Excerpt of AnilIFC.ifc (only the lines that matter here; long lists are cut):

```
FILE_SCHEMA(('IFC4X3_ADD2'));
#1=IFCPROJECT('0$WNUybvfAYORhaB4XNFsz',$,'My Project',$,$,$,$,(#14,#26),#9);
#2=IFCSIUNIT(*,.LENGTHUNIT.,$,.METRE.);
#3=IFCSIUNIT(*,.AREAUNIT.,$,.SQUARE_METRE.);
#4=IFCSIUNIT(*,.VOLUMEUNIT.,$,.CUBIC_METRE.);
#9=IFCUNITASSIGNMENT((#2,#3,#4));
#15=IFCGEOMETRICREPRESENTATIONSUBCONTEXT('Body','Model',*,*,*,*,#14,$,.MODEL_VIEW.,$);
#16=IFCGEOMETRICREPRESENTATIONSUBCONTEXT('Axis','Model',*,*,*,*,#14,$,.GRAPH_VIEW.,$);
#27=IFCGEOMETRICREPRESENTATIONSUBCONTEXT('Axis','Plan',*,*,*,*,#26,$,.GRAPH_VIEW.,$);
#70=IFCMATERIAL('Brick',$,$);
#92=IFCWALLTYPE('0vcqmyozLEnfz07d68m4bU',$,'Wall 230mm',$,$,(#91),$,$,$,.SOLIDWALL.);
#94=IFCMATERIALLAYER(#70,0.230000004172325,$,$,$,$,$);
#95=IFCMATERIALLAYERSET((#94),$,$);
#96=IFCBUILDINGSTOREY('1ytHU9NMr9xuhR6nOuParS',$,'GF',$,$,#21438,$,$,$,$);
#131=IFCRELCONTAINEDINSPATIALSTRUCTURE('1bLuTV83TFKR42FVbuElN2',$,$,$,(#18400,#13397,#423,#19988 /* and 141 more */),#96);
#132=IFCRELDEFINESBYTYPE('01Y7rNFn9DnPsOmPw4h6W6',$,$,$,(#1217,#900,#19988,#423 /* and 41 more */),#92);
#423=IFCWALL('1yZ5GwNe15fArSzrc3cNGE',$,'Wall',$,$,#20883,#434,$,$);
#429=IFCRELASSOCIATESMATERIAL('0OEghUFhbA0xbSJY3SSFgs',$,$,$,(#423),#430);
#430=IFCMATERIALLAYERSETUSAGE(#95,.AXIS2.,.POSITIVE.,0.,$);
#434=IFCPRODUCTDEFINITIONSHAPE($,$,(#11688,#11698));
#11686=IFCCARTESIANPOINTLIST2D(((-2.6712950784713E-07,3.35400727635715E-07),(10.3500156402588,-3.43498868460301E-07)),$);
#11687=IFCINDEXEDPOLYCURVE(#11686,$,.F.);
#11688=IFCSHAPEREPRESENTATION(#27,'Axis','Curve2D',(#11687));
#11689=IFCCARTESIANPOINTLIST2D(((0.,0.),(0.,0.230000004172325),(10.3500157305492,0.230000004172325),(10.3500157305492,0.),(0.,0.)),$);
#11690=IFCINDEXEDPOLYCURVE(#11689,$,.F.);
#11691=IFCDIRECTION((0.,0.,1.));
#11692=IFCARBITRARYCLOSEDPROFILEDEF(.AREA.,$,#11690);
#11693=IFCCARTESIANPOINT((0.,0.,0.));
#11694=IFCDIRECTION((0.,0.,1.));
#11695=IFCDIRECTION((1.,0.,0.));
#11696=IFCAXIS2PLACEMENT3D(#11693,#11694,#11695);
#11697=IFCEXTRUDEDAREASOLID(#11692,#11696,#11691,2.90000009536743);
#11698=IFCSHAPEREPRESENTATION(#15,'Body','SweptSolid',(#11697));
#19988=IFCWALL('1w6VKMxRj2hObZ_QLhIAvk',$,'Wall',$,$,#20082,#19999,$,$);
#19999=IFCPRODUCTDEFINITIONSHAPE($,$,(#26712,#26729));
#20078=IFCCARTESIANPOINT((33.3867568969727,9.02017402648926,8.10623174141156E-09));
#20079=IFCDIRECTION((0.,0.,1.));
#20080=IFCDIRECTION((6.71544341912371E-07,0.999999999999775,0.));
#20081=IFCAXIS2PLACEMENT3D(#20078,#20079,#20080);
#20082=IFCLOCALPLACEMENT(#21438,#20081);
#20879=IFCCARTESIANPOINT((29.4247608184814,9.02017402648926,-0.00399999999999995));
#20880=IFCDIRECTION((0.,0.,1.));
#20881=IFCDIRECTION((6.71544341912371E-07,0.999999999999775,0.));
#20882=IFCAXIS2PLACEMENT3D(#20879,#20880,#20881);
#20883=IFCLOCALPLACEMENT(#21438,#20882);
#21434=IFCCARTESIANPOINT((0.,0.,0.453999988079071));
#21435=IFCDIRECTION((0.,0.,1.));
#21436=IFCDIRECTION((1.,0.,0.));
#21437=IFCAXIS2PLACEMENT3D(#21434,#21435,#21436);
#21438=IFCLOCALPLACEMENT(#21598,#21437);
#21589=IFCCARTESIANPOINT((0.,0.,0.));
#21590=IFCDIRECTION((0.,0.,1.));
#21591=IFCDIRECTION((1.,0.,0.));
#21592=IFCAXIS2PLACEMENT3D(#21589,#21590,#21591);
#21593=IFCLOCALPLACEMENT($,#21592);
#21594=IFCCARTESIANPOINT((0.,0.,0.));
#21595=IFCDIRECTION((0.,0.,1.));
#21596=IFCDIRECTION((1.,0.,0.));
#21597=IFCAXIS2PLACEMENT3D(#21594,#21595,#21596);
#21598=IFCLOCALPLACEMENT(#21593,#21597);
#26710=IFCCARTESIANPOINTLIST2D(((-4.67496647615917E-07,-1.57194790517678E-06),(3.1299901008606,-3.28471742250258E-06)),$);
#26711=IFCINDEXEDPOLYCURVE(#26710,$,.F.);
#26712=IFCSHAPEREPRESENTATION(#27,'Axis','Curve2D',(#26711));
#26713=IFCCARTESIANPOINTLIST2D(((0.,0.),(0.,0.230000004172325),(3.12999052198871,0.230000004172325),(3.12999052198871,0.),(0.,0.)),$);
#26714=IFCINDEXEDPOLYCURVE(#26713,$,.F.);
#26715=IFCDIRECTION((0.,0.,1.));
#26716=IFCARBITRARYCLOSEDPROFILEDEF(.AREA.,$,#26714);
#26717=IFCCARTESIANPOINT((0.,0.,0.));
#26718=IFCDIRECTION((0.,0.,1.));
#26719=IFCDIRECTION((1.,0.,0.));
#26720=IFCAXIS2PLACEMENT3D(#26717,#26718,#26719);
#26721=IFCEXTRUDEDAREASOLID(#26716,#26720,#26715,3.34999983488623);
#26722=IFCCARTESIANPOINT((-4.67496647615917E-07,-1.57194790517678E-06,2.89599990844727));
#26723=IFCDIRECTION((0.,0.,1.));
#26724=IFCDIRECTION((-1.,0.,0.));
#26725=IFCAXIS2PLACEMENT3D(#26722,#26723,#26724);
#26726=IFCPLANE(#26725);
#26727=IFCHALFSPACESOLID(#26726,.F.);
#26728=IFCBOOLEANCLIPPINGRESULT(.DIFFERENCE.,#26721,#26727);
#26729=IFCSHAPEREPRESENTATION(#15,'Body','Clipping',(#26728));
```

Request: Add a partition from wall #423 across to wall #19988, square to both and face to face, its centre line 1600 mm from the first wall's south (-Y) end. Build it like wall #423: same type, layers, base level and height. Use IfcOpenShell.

```python
import numpy as np
import ifcopenshell
import ifcopenshell.api.geometry
import ifcopenshell.api.material
import ifcopenshell.api.pset
import ifcopenshell.api.root
import ifcopenshell.api.spatial
import ifcopenshell.api.type
import ifcopenshell.geom
import ifcopenshell.util.element
import ifcopenshell.util.placement
import ifcopenshell.util.representation
import ifcopenshell.util.shape
import ifcopenshell.util.unit

model = ifcopenshell.open("AnilIFC.ifc")
unit_scale = ifcopenshell.util.unit.calculate_unit_scale(model)
settings = ifcopenshell.geom.settings()
settings.set("use-world-coords", True)

start_wall = model.by_guid("1yZ5GwNe15fArSzrc3cNGE")
end_wall = model.by_guid("1w6VKMxRj2hObZ_QLhIAvk")
like = model.by_guid("1yZ5GwNe15fArSzrc3cNGE")
matrix = ifcopenshell.util.placement.get_local_placement(start_wall.ObjectPlacement)
matrix[:3, 3] *= unit_scale


def extent(element):
    """Bounding box in the first wall's axes, in metres."""
    shape = ifcopenshell.geom.create_shape(settings, element)
    points = (ifcopenshell.util.shape.get_vertices(shape.geometry) - matrix[:3, 3]) @ matrix[:3, :3]
    return points.min(axis=0), points.max(axis=0)


y_start = extent(start_wall)[0][1]
y_end = extent(end_wall)[1][1]
like_min, like_max = extent(like)
length, height = float(abs(y_end - y_start)), float(like_max[2] - like_min[2])
layer_set = ifcopenshell.util.element.get_material(like, should_skip_usage=True)
thickness = sum(layer.LayerThickness for layer in layer_set.MaterialLayers) * unit_scale

wall = ifcopenshell.api.root.create_entity(model, ifc_class="IfcWall", name="New partition")
storey = ifcopenshell.util.element.get_container(like)
ifcopenshell.api.spatial.assign_container(model, products=[wall], relating_structure=storey)
ifcopenshell.api.type.assign_type(
    model, related_objects=[wall], relating_type=ifcopenshell.util.element.get_type(like), should_map_representations=False
)
rel = ifcopenshell.api.material.assign_material(
    model, products=[wall], type="IfcMaterialLayerSetUsage", material=layer_set
)
rel.RelatingMaterial.OffsetFromReferenceLine = -thickness / 2 / unit_scale
pset = ifcopenshell.api.pset.add_pset(model, product=wall, name="Pset_WallCommon")
ifcopenshell.api.pset.edit_pset(model, pset=pset, properties={"IsExternal": False, "LoadBearing": False})

# The axis runs down the middle of the wall.
axis = ifcopenshell.api.geometry.add_axis_representation(
    model, context=ifcopenshell.util.representation.get_context(model, "Model", "Axis"), axis=[(0.0, 0.0), (length, 0.0)]
)
body = ifcopenshell.api.geometry.add_wall_representation(
    model,
    context=ifcopenshell.util.representation.get_context(model, "Model", "Body", "MODEL_VIEW"),
    length=length,
    height=height,
    thickness=thickness,
    offset=-thickness / 2,
)
for representation in (axis, body):
    ifcopenshell.api.geometry.assign_representation(model, product=wall, representation=representation)

placement = matrix @ ifcopenshell.util.placement.rotation(-90, "Z")
placement[:, 3] = matrix @ np.array([extent(start_wall)[0][0] + 1.6, y_start, like_min[2], 1.0])
ifcopenshell.api.geometry.edit_object_placement(model, product=wall, matrix=placement)

print(f"partition {length:.3f} m long, {height:.3f} m high, {thickness:.3f} m thick")

model.write("AnilIFC_v2.ifc")
```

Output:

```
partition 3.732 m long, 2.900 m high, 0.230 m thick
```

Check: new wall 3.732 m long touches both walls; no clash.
